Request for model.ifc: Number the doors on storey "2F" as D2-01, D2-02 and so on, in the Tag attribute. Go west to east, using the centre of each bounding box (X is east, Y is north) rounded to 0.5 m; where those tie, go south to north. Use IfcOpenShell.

First a look at what the model holds.

```python
import ifcopenshell
import ifcopenshell.util.element
import ifcopenshell.util.placement

model = ifcopenshell.open("model.ifc")
print(model.schema)
storey = next(s for s in model.by_type("IfcBuildingStorey") if s.Name == "2F")
doors = [e for e in ifcopenshell.util.element.get_decomposition(storey) if e.is_a("IfcDoor")]
for e in sorted(doors, key=lambda e: e.id()):
    origin = ifcopenshell.util.placement.get_local_placement(e.ObjectPlacement)[:3, 3]
    print(e.id(), e.Tag, e.Name, origin.round(2) + 0.0, sep=" | ")
```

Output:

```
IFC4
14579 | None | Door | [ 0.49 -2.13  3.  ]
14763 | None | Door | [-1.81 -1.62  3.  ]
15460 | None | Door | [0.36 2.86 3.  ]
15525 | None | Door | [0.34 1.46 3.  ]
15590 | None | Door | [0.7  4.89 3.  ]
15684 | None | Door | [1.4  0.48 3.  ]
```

```python
import ifcopenshell
import ifcopenshell.geom
import ifcopenshell.util.element
import ifcopenshell.util.shape

model = ifcopenshell.open("model.ifc")
settings = ifcopenshell.geom.settings()
settings.set("use-world-coords", True)


def centre(element):
    shape = ifcopenshell.geom.create_shape(settings, element)
    return ifcopenshell.util.shape.get_bbox_centroid(shape.geometry)


storey = next(s for s in model.by_type("IfcBuildingStorey") if s.Name == "2F")
doors = [e for e in ifcopenshell.util.element.get_decomposition(storey) if e.is_a("IfcDoor")]

# Insertion points can sit at a corner or the storey origin, so sort by the geometry (in metres).
centres = {e: centre(e) for e in doors}
doors.sort(key=lambda e: (round(centres[e][0] / 0.5), centres[e][1]))

for i, e in enumerate(doors, start=1):
    number = f"D2-{i:02d}"
    e.Tag = number
    print(e.id(), number)

model.write("model_edited.ifc")
```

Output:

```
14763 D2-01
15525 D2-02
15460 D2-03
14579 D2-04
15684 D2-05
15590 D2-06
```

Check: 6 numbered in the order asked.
